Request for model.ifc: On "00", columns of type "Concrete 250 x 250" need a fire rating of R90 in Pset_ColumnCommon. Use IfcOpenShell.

First a look at what the model holds.

```python
import ifcopenshell
import ifcopenshell.util.element

model = ifcopenshell.open("model.ifc")
print(model.schema)
storey = next(s for s in model.by_type("IfcBuildingStorey") if s.Name == "00")
columns = [e for e in ifcopenshell.util.element.get_decomposition(storey) if e.is_a("IfcColumn")]
seen = {}
for e in columns:
    element_type = ifcopenshell.util.element.get_type(e)
    key = (element_type.Name if element_type != e and element_type else None, ifcopenshell.util.element.get_pset(e, "Pset_ColumnCommon", "FireRating"))
    seen[key] = seen.get(key, 0) + 1
for (name, value), count in sorted(seen.items(), key=str):
    print(count, "x", name, "|", value)
```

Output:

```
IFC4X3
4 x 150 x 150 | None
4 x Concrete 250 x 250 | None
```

```python
import ifcopenshell
import ifcopenshell.api.pset
import ifcopenshell.util.element

model = ifcopenshell.open("model.ifc")

storey = next(s for s in model.by_type("IfcBuildingStorey") if s.Name == "00")
columns = [e for e in ifcopenshell.util.element.get_decomposition(storey) if e.is_a("IfcColumn")]

count = 0
for e in columns:
    element_type = ifcopenshell.util.element.get_type(e)
    if element_type in (None, e) or element_type.Name != "Concrete 250 x 250":
        continue
    # add_pset returns the element's existing set when there is one.
    pset = ifcopenshell.api.pset.add_pset(model, product=e, name="Pset_ColumnCommon")
    ifcopenshell.api.pset.edit_pset(model, pset=pset, properties={"FireRating": "R90"})
    count += 1

print(count, "columns updated")

model.write("model_v2.ifc")
```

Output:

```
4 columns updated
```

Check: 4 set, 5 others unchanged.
